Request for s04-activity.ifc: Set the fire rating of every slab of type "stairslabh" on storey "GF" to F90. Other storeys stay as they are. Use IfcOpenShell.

First a look at what the model holds.

```python
import ifcopenshell
import ifcopenshell.util.element

model = ifcopenshell.open("s04-activity.ifc")
print(model.schema)
storey = next(s for s in model.by_type("IfcBuildingStorey") if s.Name == "GF")
slabs = [e for e in ifcopenshell.util.element.get_decomposition(storey) if e.is_a("IfcSlab")]
seen = {}
for e in slabs:
    element_type = ifcopenshell.util.element.get_type(e)
    key = (element_type.Name if element_type != e and element_type else None, ifcopenshell.util.element.get_pset(e, "Pset_SlabCommon", "FireRating"))
    seen[key] = seen.get(key, 0) + 1
for (name, value), count in sorted(seen.items(), key=str):
    print(count, "x", name, "|", value)
```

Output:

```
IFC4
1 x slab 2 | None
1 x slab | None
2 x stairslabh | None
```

```python
import ifcopenshell
import ifcopenshell.api.pset
import ifcopenshell.util.element

model = ifcopenshell.open("s04-activity.ifc")

storey = next(s for s in model.by_type("IfcBuildingStorey") if s.Name == "GF")
slabs = [e for e in ifcopenshell.util.element.get_decomposition(storey) if e.is_a("IfcSlab")]

count = 0
for e in slabs:
    element_type = ifcopenshell.util.element.get_type(e)
    if element_type in (None, e) or element_type.Name != "stairslabh":
        continue
    # add_pset returns the element's existing set when there is one.
    pset = ifcopenshell.api.pset.add_pset(model, product=e, name="Pset_SlabCommon")
    ifcopenshell.api.pset.edit_pset(model, pset=pset, properties={"FireRating": "F90"})
    count += 1

print(count, "slabs updated")

model.write("s04-activity_updated.ifc")
```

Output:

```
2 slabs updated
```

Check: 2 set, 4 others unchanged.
